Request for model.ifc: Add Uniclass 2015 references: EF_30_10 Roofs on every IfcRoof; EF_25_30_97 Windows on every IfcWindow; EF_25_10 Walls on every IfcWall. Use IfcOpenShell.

First a look at what the model holds.

```python
import ifcopenshell

model = ifcopenshell.open("model.ifc")
print(model.schema)
print("classifications:", [c.Name for c in model.by_type("IfcClassification")])
for ifc_class in ("IfcDoor", "IfcRoof", "IfcStair", "IfcWall", "IfcWindow"):
    print(ifc_class, len(model.by_type(ifc_class)))
```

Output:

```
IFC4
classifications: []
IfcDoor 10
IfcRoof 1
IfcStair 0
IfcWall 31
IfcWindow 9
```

```python
import ifcopenshell
import ifcopenshell.api.classification

model = ifcopenshell.open("model.ifc")

system = ifcopenshell.api.classification.add_classification(model, classification="Uniclass 2015")

codes = {
    "IfcRoof": ("EF_30_10", "Roofs"),
    "IfcWindow": ("EF_25_30_97", "Windows"),
    "IfcWall": ("EF_25_10", "Walls"),
}
for ifc_class, (code, name) in codes.items():
    products = model.by_type(ifc_class)
    ifcopenshell.api.classification.add_reference(
        model, products=products, classification=system, identification=code, name=name
    )
    print(code, len(products))

model.write("model_rev.ifc")
```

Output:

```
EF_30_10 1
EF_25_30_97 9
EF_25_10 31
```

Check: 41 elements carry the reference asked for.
